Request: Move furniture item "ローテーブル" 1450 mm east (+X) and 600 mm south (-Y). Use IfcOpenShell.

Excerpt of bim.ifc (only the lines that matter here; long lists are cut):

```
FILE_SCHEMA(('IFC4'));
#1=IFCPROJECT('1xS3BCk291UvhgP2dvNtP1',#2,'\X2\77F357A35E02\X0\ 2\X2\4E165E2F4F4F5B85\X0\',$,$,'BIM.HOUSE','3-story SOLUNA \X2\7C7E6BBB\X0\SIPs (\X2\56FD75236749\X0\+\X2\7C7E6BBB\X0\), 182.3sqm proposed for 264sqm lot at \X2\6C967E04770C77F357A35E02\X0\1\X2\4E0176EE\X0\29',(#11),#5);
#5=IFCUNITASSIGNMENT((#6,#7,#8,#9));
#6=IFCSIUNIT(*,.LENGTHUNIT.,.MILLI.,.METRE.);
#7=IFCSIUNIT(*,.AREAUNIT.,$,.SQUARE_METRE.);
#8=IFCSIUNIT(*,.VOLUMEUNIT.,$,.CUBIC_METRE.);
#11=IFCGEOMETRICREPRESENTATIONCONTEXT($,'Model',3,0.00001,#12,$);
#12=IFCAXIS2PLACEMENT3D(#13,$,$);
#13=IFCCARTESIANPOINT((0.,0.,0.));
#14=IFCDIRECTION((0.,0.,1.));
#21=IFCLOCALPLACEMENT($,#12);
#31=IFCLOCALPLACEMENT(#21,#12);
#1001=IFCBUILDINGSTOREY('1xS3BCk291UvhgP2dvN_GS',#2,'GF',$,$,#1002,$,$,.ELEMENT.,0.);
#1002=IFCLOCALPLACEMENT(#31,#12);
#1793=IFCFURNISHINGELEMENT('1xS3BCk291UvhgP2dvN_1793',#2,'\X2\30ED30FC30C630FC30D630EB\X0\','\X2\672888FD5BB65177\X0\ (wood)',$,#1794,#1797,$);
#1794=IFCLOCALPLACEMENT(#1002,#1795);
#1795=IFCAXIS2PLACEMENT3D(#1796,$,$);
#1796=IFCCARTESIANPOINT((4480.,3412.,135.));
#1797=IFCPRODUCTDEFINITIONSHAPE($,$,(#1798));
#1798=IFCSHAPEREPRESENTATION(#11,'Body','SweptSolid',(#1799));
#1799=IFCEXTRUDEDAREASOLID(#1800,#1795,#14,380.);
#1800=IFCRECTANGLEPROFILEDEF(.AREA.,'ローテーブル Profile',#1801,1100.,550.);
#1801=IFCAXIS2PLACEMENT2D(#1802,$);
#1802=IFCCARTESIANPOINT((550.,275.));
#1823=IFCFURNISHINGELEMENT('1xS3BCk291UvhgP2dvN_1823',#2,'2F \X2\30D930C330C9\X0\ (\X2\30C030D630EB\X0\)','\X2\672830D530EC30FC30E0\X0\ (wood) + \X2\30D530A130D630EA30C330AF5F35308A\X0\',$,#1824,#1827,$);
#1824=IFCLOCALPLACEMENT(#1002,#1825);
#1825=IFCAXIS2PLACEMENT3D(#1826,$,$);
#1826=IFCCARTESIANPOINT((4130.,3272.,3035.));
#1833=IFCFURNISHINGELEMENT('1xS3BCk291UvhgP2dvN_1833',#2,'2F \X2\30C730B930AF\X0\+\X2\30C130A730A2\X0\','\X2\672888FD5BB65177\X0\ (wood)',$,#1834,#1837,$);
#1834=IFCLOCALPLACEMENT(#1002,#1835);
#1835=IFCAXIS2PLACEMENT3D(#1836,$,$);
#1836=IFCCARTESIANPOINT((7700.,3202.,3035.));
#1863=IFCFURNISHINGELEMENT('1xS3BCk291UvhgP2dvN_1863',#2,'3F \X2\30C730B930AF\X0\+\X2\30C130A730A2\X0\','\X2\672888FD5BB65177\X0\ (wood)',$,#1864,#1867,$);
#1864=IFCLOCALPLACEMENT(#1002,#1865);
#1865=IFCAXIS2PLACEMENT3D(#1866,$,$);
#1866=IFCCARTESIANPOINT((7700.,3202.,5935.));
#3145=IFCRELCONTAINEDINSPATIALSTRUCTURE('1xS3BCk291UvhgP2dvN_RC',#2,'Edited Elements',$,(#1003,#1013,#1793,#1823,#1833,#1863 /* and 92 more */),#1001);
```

```python
import ifcopenshell
import ifcopenshell.api.geometry
import ifcopenshell.util.placement
import ifcopenshell.util.unit

model = ifcopenshell.open("bim.ifc")
unit_scale = ifcopenshell.util.unit.calculate_unit_scale(model)

item = model.by_id(1793)
matrix = ifcopenshell.util.placement.get_local_placement(item.ObjectPlacement)
matrix[0, 3] += 1.45 / unit_scale
matrix[1, 3] -= 0.6 / unit_scale
ifcopenshell.api.geometry.edit_object_placement(model, product=item, matrix=matrix, is_si=False)

print(ifcopenshell.util.placement.get_local_placement(item.ObjectPlacement).round(3) + 0.0)

model.write("bim_updated.ifc")
```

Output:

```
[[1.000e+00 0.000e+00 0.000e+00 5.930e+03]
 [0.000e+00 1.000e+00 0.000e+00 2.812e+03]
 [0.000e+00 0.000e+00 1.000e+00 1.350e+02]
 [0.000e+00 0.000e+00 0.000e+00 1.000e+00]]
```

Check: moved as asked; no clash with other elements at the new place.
